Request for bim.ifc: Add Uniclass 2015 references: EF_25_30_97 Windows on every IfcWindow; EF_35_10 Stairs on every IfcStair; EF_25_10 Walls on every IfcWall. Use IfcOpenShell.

First a look at what the model holds.

```python
import ifcopenshell

model = ifcopenshell.open("bim.ifc")
print(model.schema)
print("classifications:", [c.Name for c in model.by_type("IfcClassification")])
for ifc_class in ("IfcDoor", "IfcRoof", "IfcStair", "IfcWall", "IfcWindow"):
    print(ifc_class, len(model.by_type(ifc_class)))
```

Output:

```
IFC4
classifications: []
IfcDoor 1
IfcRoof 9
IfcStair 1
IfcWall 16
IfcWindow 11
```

```python
import ifcopenshell
import ifcopenshell.api.classification

model = ifcopenshell.open("bim.ifc")

system = ifcopenshell.api.classification.add_classification(model, classification="Uniclass 2015")

codes = {
    "IfcWindow": ("EF_25_30_97", "Windows"),
    "IfcStair": ("EF_35_10", "Stairs"),
    "IfcWall": ("EF_25_10", "Walls"),
}
for ifc_class, (code, name) in codes.items():
    products = model.by_type(ifc_class)
    ifcopenshell.api.classification.add_reference(
        model, products=products, classification=system, identification=code, name=name
    )
    print(code, len(products))

model.write("bim_edited.ifc")
```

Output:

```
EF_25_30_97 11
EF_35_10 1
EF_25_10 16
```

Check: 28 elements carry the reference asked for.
